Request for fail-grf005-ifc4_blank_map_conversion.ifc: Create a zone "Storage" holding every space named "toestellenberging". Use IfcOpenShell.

First a look at what the model holds.

```python
import ifcopenshell

model = ifcopenshell.open("fail-grf005-ifc4_blank_map_conversion.ifc")
print(model.schema)
seen = {}
for space in model.by_type("IfcSpace"):
    seen[space.LongName] = seen.get(space.LongName, 0) + 1
for name, count in sorted(seen.items(), key=str):
    print(count, "x", name)
print("zones:", [z.Name for z in model.by_type("IfcZone")][:20])
```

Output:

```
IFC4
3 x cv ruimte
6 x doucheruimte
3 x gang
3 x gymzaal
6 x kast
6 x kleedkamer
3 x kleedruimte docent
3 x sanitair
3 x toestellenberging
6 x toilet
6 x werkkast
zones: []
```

```python
import ifcopenshell
import ifcopenshell.api.group
import ifcopenshell.api.root

model = ifcopenshell.open("fail-grf005-ifc4_blank_map_conversion.ifc")

names = {"toestellenberging"}
spaces = [s for s in model.by_type("IfcSpace") if s.LongName in names]

zone = ifcopenshell.api.root.create_entity(model, ifc_class="IfcZone", name="Storage")
ifcopenshell.api.group.assign_group(model, products=spaces, group=zone)
print(len(spaces), "spaces in", zone.Name)

model.write("fail-grf005-ifc4_blank_map_conversion-out.ifc")
```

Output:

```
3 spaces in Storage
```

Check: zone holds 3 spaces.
